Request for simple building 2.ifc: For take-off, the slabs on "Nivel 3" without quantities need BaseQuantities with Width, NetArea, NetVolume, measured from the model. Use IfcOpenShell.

First a look at what the model holds.

```python
import ifcopenshell
import ifcopenshell.util.element
import ifcopenshell.util.unit

model = ifcopenshell.open("simple building 2.ifc")
print(model.schema)
for unit_type in ("LENGTHUNIT", "AREAUNIT", "VOLUMEUNIT"):
    print(unit_type, ifcopenshell.util.unit.calculate_unit_scale(model, unit_type))
storey = next(s for s in model.by_type("IfcBuildingStorey") if s.Name == "Nivel 3")
slabs = [e for e in ifcopenshell.util.element.get_decomposition(storey) if e.is_a("IfcSlab")]
for e in sorted(slabs, key=lambda e: e.id()):
    print(e.id(), e.is_a(), e.Name, list(ifcopenshell.util.element.get_psets(e, qtos_only=True)), sep=" | ")
```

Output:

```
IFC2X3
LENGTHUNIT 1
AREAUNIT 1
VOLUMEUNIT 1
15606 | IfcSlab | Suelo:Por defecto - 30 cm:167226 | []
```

```python
import ifcopenshell
import ifcopenshell.api.pset
import ifcopenshell.geom
import ifcopenshell.util.element
import ifcopenshell.util.shape
import ifcopenshell.util.unit

model = ifcopenshell.open("simple building 2.ifc")
unit_scale = ifcopenshell.util.unit.calculate_unit_scale(model)
area_scale = ifcopenshell.util.unit.calculate_unit_scale(model, "AREAUNIT")
volume_scale = ifcopenshell.util.unit.calculate_unit_scale(model, "VOLUMEUNIT")
settings = ifcopenshell.geom.settings()

storey = next(s for s in model.by_type("IfcBuildingStorey") if s.Name == "Nivel 3")
slabs = [e for e in ifcopenshell.util.element.get_decomposition(storey) if e.is_a("IfcSlab")]

for e in sorted(slabs, key=lambda e: e.id()):
    if ifcopenshell.util.element.get_psets(e, qtos_only=True, should_inherit=False):
        continue
    # Geometry comes back in metres, in the element's own axes.
    shape = ifcopenshell.geom.create_shape(settings, e)
    values = {
        "Width": ifcopenshell.util.shape.get_z(shape.geometry) / unit_scale,
        "NetArea": ifcopenshell.util.shape.get_footprint_area(shape.geometry) / area_scale,
        "NetVolume": ifcopenshell.util.shape.get_volume(shape.geometry) / volume_scale,
    }
    qto = ifcopenshell.api.pset.add_qto(model, product=e, name="BaseQuantities")
    ifcopenshell.api.pset.edit_qto(model, qto=qto, properties=values)
    print(e.id(), {k: round(v, 3) for k, v in values.items()})

model.write("simple building 2_updated.ifc")
```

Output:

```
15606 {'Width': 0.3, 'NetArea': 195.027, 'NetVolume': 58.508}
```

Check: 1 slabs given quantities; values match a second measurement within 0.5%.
